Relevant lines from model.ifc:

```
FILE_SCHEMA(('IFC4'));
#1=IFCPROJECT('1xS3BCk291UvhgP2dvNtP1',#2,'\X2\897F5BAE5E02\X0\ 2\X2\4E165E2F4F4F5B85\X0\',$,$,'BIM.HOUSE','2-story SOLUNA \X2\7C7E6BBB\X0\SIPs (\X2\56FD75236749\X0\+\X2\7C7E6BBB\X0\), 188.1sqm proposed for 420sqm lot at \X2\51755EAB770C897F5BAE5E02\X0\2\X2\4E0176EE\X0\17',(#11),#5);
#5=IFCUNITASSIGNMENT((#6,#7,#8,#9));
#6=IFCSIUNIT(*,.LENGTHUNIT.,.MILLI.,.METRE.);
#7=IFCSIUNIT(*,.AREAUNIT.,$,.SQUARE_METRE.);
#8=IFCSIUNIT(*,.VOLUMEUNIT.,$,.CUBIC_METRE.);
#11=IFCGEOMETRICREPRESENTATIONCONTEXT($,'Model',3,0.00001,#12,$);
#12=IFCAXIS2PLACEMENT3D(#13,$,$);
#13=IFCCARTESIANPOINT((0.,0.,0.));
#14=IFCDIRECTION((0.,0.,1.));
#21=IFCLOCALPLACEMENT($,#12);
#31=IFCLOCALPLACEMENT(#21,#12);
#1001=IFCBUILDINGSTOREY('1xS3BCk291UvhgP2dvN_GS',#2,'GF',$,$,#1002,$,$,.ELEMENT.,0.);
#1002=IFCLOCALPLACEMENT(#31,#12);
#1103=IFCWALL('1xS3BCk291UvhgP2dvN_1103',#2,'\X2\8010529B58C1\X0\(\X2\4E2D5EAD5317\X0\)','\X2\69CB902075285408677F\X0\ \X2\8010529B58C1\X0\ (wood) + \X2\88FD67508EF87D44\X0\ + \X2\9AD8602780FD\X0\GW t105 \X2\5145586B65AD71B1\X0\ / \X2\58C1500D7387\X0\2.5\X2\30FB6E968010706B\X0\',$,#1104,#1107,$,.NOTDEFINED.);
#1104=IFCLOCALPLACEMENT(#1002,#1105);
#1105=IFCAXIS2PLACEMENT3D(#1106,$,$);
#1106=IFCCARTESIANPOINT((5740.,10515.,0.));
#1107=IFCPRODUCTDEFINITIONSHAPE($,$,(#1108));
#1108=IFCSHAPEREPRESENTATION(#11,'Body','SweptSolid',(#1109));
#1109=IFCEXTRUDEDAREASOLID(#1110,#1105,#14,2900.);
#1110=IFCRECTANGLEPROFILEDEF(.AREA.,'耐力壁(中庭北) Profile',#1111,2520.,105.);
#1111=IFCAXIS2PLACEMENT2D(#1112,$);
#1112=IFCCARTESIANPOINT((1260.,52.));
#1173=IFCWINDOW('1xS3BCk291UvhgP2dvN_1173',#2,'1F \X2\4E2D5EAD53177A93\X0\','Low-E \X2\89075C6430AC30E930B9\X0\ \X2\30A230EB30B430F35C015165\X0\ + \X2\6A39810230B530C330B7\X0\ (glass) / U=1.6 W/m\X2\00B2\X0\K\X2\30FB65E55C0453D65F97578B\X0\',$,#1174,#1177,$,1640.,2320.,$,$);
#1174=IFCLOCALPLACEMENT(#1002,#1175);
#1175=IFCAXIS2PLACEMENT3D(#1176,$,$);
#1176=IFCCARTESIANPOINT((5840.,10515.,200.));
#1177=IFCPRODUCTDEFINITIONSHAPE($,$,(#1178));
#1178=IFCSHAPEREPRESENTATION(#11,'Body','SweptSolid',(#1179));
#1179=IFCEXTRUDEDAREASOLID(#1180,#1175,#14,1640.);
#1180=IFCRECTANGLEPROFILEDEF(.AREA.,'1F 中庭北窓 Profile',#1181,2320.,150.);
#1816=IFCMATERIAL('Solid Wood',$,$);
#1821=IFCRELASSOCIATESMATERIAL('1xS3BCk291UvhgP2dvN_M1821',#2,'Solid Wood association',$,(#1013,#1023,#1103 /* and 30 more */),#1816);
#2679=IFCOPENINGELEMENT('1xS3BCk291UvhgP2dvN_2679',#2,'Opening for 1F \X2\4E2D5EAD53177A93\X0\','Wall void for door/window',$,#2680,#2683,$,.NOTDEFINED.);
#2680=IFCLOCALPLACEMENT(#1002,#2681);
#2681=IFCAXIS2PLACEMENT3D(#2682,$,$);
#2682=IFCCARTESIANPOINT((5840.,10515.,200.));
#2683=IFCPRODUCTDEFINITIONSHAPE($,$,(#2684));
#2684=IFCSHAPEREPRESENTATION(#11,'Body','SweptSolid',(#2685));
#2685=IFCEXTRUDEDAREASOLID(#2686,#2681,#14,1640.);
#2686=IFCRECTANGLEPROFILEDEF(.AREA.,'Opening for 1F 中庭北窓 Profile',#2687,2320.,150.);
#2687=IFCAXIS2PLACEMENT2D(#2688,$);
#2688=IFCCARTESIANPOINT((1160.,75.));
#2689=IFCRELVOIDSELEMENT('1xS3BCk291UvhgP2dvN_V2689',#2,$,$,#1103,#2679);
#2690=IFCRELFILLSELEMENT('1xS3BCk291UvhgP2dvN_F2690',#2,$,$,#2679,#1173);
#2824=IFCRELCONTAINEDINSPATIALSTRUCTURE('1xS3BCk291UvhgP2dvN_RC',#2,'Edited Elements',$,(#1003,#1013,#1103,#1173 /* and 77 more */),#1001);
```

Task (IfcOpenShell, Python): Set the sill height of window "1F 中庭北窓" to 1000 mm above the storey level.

```python
import numpy as np
import ifcopenshell
import ifcopenshell.api.geometry
import ifcopenshell.geom
import ifcopenshell.util.element
import ifcopenshell.util.placement
import ifcopenshell.util.shape
import ifcopenshell.util.unit

model = ifcopenshell.open("model.ifc")
unit_scale = ifcopenshell.util.unit.calculate_unit_scale(model)

window = model.by_guid("1xS3BCk291UvhgP2dvN_1173")
opening = window.FillsVoids[0].RelatingOpeningElement
storey = ifcopenshell.util.element.get_container(window, ifc_class="IfcBuildingStorey")
level = ifcopenshell.util.placement.get_local_placement(storey.ObjectPlacement)[2, 3]

# The opening's origin need not be at the sill, so measure its lowest point.
shape = ifcopenshell.geom.create_shape(ifcopenshell.geom.settings(), opening)
bottom = ifcopenshell.util.shape.get_shape_bottom_elevation(shape, shape.geometry) / unit_scale
dz = level + 1 / unit_scale - bottom

shift = np.array([0.0, 0.0, dz])
# The window is not placed relative to its opening, so move both.
for product in (opening, window):
    matrix = ifcopenshell.util.placement.get_local_placement(product.ObjectPlacement)
    matrix[:3, 3] += shift
    ifcopenshell.api.geometry.edit_object_placement(model, product=product, matrix=matrix, is_si=False)

print(f"moved by {dz * unit_scale:+.3f} m")

model.write("model_edited.ifc")
```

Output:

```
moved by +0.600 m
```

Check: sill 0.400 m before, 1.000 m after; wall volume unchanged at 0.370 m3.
